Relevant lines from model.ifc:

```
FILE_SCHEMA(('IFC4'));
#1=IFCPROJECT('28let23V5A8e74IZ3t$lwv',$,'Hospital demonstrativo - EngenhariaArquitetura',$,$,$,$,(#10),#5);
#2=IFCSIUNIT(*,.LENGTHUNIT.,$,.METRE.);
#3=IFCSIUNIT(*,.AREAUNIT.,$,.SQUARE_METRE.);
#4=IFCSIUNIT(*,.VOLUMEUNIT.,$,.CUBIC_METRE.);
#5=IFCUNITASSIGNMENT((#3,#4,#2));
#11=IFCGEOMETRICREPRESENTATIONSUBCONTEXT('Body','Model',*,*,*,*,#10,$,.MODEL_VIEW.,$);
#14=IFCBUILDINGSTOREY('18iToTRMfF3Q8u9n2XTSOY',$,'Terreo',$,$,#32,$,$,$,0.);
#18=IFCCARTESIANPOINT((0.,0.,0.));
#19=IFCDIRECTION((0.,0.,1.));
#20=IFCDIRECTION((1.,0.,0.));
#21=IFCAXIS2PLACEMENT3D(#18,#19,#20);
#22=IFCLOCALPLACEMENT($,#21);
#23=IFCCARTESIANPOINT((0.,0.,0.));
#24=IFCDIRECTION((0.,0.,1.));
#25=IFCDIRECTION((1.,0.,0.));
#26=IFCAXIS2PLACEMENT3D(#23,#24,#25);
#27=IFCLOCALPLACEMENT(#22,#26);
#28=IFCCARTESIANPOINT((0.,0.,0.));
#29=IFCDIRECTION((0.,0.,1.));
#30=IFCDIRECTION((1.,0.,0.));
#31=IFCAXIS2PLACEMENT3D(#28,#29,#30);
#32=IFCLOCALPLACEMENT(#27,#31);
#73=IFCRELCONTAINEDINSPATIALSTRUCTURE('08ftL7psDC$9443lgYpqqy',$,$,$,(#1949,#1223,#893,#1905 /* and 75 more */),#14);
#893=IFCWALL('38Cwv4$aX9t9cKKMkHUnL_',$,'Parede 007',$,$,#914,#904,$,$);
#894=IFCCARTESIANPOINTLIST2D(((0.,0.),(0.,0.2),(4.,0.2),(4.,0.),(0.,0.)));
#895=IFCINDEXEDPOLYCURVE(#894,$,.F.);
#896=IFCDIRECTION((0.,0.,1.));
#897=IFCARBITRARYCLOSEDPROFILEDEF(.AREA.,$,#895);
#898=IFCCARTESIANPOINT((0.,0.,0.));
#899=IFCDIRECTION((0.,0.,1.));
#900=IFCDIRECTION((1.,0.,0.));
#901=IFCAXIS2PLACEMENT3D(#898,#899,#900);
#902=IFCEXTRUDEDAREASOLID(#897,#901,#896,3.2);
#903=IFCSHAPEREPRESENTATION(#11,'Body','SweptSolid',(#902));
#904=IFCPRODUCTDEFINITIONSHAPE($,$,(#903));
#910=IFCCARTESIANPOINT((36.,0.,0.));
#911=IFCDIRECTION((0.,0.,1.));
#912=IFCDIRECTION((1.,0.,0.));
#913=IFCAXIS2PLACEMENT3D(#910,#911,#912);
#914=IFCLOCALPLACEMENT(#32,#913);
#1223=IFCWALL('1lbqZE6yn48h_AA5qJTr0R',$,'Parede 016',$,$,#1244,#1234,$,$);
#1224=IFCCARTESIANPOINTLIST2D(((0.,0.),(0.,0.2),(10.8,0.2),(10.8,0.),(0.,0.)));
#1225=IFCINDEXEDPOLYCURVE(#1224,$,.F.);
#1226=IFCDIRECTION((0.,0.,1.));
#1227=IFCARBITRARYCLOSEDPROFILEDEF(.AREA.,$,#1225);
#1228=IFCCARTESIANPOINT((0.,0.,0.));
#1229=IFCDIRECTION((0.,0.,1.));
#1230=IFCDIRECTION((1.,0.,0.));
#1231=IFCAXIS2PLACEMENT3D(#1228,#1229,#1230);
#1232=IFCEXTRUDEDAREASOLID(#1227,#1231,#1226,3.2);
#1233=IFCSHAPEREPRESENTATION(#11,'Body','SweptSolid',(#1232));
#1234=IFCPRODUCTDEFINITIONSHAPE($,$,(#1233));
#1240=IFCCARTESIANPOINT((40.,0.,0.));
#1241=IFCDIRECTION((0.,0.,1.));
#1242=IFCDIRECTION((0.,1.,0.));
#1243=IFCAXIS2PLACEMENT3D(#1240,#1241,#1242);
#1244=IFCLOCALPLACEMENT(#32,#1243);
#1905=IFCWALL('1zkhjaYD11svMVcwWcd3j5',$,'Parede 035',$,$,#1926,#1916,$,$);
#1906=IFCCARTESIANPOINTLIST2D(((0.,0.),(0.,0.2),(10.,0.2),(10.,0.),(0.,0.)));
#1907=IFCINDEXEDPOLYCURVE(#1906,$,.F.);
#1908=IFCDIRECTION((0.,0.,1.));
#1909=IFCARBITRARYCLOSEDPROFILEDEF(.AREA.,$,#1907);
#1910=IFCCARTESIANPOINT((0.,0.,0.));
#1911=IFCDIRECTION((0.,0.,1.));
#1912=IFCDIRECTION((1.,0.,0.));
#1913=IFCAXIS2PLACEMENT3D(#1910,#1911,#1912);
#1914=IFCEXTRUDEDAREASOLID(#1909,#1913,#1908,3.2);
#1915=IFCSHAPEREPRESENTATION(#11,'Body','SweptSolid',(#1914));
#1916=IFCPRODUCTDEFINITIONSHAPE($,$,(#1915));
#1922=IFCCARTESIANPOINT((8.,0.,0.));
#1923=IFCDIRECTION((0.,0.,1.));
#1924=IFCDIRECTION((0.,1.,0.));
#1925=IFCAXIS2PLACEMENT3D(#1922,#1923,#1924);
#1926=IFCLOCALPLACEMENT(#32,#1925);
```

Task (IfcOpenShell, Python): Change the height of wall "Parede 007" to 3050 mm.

```python
import ifcopenshell
import ifcopenshell.geom
import ifcopenshell.util.representation
import ifcopenshell.util.shape
import ifcopenshell.util.unit

model = ifcopenshell.open("model.ifc")
unit_scale = ifcopenshell.util.unit.calculate_unit_scale(model)
settings = ifcopenshell.geom.settings()


def volume(element):
    """Net volume in cubic metres, openings subtracted."""
    shape = ifcopenshell.geom.create_shape(settings, element)
    return ifcopenshell.util.shape.get_volume(shape.geometry)


wall = model.by_guid("38Cwv4$aX9t9cKKMkHUnL_")
before = volume(wall)

body = ifcopenshell.util.representation.get_representation(wall, "Model", "Body")
solid = body.Items[0]
old_height = solid.Depth
solid.Depth = 3.05 / unit_scale
after = volume(wall)

print(f"height {old_height:g} -> {solid.Depth:g}, volume {before:.3f} -> {after:.3f} m3")

model.write("model-out.ifc")
```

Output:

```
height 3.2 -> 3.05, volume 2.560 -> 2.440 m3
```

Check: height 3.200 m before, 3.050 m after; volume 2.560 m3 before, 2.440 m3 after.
